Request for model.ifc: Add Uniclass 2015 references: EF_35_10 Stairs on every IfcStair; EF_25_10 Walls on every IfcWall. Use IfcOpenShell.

First a look at what the model holds.

```python
import ifcopenshell

model = ifcopenshell.open("model.ifc")
print(model.schema)
print("classifications:", [c.Name for c in model.by_type("IfcClassification")])
for ifc_class in ("IfcDoor", "IfcRoof", "IfcStair", "IfcWall", "IfcWindow"):
    print(ifc_class, len(model.by_type(ifc_class)))
```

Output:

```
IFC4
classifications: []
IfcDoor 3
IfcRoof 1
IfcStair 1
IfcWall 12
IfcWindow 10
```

```python
import ifcopenshell
import ifcopenshell.api.classification

model = ifcopenshell.open("model.ifc")

system = ifcopenshell.api.classification.add_classification(model, classification="Uniclass 2015")

codes = {
    "IfcStair": ("EF_35_10", "Stairs"),
    "IfcWall": ("EF_25_10", "Walls"),
}
for ifc_class, (code, name) in codes.items():
    products = model.by_type(ifc_class)
    ifcopenshell.api.classification.add_reference(
        model, products=products, classification=system, identification=code, name=name
    )
    print(code, len(products))

model.write("model_v2.ifc")
```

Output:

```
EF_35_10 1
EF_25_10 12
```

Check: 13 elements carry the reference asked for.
